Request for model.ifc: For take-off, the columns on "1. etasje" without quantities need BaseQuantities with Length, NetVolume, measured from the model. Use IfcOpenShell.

First a look at what the model holds.

```python
import ifcopenshell
import ifcopenshell.util.element
import ifcopenshell.util.unit

model = ifcopenshell.open("model.ifc")
print(model.schema)
for unit_type in ("LENGTHUNIT", "AREAUNIT", "VOLUMEUNIT"):
    print(unit_type, ifcopenshell.util.unit.calculate_unit_scale(model, unit_type))
storey = next(s for s in model.by_type("IfcBuildingStorey") if s.Name == "1. etasje")
columns = [e for e in ifcopenshell.util.element.get_decomposition(storey) if e.is_a("IfcColumn")]
for e in sorted(columns, key=lambda e: e.id()):
    print(e.id(), e.is_a(), e.Name, list(ifcopenshell.util.element.get_psets(e, qtos_only=True)), sep=" | ")
```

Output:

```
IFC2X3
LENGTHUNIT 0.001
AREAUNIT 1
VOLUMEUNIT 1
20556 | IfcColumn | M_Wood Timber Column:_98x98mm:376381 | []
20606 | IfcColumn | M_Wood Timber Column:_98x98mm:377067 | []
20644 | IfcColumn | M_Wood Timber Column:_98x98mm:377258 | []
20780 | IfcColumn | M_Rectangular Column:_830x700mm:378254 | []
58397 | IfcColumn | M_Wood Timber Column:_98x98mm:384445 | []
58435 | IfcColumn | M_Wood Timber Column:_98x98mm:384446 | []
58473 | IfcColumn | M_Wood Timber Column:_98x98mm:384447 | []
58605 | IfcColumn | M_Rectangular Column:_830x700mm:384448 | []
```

```python
import ifcopenshell
import ifcopenshell.api.pset
import ifcopenshell.geom
import ifcopenshell.util.element
import ifcopenshell.util.shape
import ifcopenshell.util.unit

model = ifcopenshell.open("model.ifc")
unit_scale = ifcopenshell.util.unit.calculate_unit_scale(model)
volume_scale = ifcopenshell.util.unit.calculate_unit_scale(model, "VOLUMEUNIT")
settings = ifcopenshell.geom.settings()

storey = next(s for s in model.by_type("IfcBuildingStorey") if s.Name == "1. etasje")
columns = [e for e in ifcopenshell.util.element.get_decomposition(storey) if e.is_a("IfcColumn")]

for e in sorted(columns, key=lambda e: e.id()):
    if ifcopenshell.util.element.get_psets(e, qtos_only=True, should_inherit=False):
        continue
    # Geometry comes back in metres, in the element's own axes.
    shape = ifcopenshell.geom.create_shape(settings, e)
    values = {
        "Length": ifcopenshell.util.shape.get_z(shape.geometry) / unit_scale,
        "NetVolume": ifcopenshell.util.shape.get_volume(shape.geometry) / volume_scale,
    }
    qto = ifcopenshell.api.pset.add_qto(model, product=e, name="BaseQuantities")
    ifcopenshell.api.pset.edit_qto(model, qto=qto, properties=values)
    print(e.id(), {k: round(v, 3) for k, v in values.items()})

model.write("model_edited.ifc")
```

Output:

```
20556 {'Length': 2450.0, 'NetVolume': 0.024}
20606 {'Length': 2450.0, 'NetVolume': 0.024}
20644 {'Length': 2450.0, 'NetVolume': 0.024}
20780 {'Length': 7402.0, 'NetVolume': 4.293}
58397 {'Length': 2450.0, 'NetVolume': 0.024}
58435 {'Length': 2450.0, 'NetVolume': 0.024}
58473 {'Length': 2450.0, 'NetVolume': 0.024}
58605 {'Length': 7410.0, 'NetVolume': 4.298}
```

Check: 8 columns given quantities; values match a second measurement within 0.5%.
